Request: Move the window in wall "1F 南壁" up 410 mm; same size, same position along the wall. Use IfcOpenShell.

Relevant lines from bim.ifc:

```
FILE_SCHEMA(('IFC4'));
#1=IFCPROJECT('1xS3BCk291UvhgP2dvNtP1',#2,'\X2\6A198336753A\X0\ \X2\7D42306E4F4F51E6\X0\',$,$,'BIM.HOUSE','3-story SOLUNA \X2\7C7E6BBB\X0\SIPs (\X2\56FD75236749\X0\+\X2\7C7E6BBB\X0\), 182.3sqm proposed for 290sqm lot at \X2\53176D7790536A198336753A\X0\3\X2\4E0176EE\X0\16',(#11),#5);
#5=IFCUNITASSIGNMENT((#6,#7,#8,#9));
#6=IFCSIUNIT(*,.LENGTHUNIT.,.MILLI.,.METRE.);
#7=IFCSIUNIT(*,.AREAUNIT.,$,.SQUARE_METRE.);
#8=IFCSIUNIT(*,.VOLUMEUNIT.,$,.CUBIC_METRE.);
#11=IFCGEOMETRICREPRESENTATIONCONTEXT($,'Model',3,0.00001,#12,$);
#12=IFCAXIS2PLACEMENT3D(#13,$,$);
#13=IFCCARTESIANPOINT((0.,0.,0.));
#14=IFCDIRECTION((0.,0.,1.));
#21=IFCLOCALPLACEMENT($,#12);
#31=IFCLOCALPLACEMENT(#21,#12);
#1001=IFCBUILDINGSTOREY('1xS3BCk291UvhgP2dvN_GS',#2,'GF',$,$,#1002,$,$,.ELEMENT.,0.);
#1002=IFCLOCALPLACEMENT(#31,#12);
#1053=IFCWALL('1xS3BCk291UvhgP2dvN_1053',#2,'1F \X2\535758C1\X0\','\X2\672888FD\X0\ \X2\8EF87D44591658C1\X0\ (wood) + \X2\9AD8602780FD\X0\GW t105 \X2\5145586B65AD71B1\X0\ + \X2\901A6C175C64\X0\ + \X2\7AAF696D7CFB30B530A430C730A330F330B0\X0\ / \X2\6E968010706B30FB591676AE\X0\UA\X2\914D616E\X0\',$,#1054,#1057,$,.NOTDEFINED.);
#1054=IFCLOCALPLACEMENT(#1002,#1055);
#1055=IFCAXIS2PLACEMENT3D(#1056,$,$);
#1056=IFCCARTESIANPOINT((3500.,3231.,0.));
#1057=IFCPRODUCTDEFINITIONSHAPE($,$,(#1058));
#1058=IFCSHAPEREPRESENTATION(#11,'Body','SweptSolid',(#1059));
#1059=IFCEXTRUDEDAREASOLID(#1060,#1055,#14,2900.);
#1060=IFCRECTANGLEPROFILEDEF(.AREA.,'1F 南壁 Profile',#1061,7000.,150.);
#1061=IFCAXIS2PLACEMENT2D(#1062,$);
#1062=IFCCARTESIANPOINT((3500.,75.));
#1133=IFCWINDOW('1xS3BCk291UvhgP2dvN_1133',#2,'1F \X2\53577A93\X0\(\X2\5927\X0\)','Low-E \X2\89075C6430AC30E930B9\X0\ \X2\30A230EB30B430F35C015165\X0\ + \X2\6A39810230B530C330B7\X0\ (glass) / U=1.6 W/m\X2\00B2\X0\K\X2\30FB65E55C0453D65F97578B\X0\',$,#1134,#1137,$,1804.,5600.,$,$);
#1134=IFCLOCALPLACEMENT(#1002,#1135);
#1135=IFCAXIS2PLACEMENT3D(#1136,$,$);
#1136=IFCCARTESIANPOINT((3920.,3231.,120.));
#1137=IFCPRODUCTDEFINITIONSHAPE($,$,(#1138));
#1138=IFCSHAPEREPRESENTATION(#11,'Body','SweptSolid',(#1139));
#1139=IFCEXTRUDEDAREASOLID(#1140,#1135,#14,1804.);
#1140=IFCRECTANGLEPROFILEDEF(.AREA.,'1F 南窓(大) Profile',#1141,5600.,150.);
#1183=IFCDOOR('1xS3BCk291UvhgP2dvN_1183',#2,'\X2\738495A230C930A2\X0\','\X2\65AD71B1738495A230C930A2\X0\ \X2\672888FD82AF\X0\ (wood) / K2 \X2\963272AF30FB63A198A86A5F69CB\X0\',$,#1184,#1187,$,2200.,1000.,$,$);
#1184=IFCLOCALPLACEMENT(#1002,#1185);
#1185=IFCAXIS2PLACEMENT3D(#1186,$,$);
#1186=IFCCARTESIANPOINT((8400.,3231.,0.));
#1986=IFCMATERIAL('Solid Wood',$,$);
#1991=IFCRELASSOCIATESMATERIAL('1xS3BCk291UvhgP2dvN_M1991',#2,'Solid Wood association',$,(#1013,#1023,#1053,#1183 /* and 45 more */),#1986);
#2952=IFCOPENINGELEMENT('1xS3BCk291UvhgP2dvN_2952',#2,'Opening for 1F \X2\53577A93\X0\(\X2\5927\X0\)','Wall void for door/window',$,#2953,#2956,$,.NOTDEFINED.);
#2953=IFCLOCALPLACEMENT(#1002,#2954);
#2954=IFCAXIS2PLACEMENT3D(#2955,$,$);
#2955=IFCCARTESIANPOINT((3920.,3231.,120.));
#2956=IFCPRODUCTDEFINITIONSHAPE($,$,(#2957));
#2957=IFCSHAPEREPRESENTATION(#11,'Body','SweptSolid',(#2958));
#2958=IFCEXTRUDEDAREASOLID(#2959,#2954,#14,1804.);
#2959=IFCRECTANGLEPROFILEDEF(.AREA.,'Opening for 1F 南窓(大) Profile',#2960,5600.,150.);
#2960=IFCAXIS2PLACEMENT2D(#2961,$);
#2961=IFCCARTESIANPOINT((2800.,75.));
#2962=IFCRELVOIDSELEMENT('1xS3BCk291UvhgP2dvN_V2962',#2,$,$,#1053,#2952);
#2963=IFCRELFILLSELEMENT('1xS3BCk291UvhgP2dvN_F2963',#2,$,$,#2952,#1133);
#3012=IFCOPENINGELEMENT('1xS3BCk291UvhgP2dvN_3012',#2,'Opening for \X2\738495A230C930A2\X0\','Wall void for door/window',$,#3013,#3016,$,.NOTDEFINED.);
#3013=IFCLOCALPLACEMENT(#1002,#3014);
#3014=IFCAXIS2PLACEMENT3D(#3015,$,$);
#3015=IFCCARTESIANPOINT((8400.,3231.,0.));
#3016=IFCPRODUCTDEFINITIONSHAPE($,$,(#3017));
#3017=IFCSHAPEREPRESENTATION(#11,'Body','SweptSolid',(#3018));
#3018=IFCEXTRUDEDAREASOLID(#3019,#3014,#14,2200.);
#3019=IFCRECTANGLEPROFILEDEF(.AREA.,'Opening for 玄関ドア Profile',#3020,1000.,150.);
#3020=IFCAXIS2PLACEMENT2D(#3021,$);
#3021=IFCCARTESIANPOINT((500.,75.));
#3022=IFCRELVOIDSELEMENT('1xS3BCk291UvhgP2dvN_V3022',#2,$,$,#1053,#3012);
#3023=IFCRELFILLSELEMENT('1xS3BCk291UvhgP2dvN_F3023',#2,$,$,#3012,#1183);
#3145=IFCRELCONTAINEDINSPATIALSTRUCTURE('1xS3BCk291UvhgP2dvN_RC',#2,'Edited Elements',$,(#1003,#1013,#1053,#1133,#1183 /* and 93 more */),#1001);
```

```python
import numpy as np
import ifcopenshell
import ifcopenshell.api.geometry
import ifcopenshell.util.placement
import ifcopenshell.util.unit

model = ifcopenshell.open("bim.ifc")
unit_scale = ifcopenshell.util.unit.calculate_unit_scale(model)

window = model.by_guid("1xS3BCk291UvhgP2dvN_1133")
opening = window.FillsVoids[0].RelatingOpeningElement
dz = 0.41 / unit_scale

shift = np.array([0.0, 0.0, dz])
# The window is not placed relative to its opening, so move both.
for product in (opening, window):
    matrix = ifcopenshell.util.placement.get_local_placement(product.ObjectPlacement)
    matrix[:3, 3] += shift
    ifcopenshell.api.geometry.edit_object_placement(model, product=product, matrix=matrix, is_si=False)

print(f"moved by {dz * unit_scale:+.3f} m")

model.write("bim-out.ifc")
```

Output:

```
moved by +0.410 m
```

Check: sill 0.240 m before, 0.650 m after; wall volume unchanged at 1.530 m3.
